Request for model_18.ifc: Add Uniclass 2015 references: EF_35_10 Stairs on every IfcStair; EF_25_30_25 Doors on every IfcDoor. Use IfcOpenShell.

First a look at what the model holds.

```python
import ifcopenshell

model = ifcopenshell.open("model_18.ifc")
print(model.schema)
print("classifications:", [c.Name for c in model.by_type("IfcClassification")])
for ifc_class in ("IfcDoor", "IfcRoof", "IfcStair", "IfcWall", "IfcWindow"):
    print(ifc_class, len(model.by_type(ifc_class)))
```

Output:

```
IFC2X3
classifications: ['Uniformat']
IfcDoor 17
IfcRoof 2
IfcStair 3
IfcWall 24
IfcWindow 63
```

```python
import ifcopenshell
import ifcopenshell.api.classification

model = ifcopenshell.open("model_18.ifc")

# IFC2X3 requires Source and Edition and has no link from the project to the system.
system = model.create_entity("IfcClassification", Source="NBS", Edition="2015", Name="Uniclass 2015")

codes = {
    "IfcStair": ("EF_35_10", "Stairs"),
    "IfcDoor": ("EF_25_30_25", "Doors"),
}
for ifc_class, (code, name) in codes.items():
    products = model.by_type(ifc_class)
    ifcopenshell.api.classification.add_reference(
        model, products=products, classification=system, identification=code, name=name
    )
    print(code, len(products))

model.write("model_18_rev.ifc")
```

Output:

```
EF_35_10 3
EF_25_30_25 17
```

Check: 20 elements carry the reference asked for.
